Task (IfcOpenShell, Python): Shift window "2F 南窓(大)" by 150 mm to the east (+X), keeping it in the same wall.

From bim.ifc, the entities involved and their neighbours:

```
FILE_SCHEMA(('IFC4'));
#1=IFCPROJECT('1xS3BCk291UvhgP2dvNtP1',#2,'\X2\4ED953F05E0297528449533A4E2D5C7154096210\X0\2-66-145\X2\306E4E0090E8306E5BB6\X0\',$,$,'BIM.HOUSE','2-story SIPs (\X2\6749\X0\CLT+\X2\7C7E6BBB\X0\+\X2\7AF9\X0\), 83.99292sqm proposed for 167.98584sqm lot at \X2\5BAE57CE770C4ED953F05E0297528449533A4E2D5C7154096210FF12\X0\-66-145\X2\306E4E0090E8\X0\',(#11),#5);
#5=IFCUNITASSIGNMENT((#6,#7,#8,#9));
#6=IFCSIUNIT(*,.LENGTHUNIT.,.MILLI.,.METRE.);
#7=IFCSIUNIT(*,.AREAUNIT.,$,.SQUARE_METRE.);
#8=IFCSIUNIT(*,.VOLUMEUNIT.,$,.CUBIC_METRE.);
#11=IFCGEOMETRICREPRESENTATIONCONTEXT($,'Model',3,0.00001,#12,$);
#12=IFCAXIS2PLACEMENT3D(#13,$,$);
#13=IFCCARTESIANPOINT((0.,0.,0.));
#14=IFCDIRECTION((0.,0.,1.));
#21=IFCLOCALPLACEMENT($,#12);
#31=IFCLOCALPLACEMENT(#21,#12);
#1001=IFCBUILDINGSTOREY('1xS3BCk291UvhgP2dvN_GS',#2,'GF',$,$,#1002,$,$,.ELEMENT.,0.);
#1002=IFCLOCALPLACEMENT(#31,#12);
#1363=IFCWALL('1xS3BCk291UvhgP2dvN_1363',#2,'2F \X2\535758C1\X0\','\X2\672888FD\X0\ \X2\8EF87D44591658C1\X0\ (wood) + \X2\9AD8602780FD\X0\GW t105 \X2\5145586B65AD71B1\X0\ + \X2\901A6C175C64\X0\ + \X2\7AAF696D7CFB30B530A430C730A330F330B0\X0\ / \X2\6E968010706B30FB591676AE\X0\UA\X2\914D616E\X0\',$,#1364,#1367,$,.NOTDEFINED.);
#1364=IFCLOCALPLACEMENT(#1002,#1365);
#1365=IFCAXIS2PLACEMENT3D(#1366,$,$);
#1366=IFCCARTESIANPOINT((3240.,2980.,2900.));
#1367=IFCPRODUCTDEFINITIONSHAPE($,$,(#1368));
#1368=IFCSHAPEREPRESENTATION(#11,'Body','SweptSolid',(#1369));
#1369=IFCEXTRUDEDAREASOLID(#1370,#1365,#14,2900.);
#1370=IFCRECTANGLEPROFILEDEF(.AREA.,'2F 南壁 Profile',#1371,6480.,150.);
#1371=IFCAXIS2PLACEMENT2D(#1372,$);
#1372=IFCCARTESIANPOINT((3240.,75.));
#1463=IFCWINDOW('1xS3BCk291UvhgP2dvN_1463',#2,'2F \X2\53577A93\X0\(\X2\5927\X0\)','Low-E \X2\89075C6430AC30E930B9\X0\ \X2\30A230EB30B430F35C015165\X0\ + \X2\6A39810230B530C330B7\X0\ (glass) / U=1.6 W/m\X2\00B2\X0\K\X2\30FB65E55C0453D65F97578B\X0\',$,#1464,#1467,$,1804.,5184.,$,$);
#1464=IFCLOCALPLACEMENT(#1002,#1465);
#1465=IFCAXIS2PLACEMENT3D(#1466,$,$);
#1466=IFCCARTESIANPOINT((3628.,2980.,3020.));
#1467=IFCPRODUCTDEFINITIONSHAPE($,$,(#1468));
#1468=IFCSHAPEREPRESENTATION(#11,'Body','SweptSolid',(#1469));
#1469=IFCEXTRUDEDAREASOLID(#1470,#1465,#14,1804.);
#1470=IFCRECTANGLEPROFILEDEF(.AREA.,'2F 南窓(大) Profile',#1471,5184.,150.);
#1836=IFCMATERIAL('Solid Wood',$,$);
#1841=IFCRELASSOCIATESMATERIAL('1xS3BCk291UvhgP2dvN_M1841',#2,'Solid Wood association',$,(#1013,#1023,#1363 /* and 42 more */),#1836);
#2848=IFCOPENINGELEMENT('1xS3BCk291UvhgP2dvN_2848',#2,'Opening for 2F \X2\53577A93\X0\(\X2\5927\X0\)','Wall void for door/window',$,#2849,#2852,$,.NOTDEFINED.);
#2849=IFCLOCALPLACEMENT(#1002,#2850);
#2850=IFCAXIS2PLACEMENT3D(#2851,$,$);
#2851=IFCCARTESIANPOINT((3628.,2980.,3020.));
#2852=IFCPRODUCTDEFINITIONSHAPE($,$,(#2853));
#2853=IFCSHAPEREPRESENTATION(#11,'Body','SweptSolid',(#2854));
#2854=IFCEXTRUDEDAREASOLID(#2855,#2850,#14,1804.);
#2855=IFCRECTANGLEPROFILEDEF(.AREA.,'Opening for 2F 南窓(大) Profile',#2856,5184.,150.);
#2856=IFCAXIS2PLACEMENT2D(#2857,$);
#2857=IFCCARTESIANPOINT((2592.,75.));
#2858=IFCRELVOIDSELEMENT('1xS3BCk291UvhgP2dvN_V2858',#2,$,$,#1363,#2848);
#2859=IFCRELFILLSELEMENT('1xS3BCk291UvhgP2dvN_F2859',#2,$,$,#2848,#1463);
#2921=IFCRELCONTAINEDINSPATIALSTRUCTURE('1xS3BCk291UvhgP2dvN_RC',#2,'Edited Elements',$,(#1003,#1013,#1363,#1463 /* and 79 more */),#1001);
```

```python
import ifcopenshell
import ifcopenshell.api.geometry
import ifcopenshell.util.placement
import ifcopenshell.util.unit

model = ifcopenshell.open("bim.ifc")
unit_scale = ifcopenshell.util.unit.calculate_unit_scale(model)

window = model.by_id(1463)
opening = window.FillsVoids[0].RelatingOpeningElement
wall = opening.VoidsElements[0].RelatingBuildingElement

wall_matrix = ifcopenshell.util.placement.get_local_placement(wall.ObjectPlacement)
shift = wall_matrix[:3, 0] * 0.15 / unit_scale
before = ifcopenshell.util.placement.get_local_placement(window.ObjectPlacement)[:3, 3].copy()

# The window is not placed relative to its opening, so move both.
for product in (opening, window):
    matrix = ifcopenshell.util.placement.get_local_placement(product.ObjectPlacement)
    matrix[:3, 3] += shift
    ifcopenshell.api.geometry.edit_object_placement(model, product=product, matrix=matrix, is_si=False)

after = ifcopenshell.util.placement.get_local_placement(window.ObjectPlacement)[:3, 3]
print("window moved by", (after - before).round(3) + 0.0)

model.write("bim_edited.ifc")
```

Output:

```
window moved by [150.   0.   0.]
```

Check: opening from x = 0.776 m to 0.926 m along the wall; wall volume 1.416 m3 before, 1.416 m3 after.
